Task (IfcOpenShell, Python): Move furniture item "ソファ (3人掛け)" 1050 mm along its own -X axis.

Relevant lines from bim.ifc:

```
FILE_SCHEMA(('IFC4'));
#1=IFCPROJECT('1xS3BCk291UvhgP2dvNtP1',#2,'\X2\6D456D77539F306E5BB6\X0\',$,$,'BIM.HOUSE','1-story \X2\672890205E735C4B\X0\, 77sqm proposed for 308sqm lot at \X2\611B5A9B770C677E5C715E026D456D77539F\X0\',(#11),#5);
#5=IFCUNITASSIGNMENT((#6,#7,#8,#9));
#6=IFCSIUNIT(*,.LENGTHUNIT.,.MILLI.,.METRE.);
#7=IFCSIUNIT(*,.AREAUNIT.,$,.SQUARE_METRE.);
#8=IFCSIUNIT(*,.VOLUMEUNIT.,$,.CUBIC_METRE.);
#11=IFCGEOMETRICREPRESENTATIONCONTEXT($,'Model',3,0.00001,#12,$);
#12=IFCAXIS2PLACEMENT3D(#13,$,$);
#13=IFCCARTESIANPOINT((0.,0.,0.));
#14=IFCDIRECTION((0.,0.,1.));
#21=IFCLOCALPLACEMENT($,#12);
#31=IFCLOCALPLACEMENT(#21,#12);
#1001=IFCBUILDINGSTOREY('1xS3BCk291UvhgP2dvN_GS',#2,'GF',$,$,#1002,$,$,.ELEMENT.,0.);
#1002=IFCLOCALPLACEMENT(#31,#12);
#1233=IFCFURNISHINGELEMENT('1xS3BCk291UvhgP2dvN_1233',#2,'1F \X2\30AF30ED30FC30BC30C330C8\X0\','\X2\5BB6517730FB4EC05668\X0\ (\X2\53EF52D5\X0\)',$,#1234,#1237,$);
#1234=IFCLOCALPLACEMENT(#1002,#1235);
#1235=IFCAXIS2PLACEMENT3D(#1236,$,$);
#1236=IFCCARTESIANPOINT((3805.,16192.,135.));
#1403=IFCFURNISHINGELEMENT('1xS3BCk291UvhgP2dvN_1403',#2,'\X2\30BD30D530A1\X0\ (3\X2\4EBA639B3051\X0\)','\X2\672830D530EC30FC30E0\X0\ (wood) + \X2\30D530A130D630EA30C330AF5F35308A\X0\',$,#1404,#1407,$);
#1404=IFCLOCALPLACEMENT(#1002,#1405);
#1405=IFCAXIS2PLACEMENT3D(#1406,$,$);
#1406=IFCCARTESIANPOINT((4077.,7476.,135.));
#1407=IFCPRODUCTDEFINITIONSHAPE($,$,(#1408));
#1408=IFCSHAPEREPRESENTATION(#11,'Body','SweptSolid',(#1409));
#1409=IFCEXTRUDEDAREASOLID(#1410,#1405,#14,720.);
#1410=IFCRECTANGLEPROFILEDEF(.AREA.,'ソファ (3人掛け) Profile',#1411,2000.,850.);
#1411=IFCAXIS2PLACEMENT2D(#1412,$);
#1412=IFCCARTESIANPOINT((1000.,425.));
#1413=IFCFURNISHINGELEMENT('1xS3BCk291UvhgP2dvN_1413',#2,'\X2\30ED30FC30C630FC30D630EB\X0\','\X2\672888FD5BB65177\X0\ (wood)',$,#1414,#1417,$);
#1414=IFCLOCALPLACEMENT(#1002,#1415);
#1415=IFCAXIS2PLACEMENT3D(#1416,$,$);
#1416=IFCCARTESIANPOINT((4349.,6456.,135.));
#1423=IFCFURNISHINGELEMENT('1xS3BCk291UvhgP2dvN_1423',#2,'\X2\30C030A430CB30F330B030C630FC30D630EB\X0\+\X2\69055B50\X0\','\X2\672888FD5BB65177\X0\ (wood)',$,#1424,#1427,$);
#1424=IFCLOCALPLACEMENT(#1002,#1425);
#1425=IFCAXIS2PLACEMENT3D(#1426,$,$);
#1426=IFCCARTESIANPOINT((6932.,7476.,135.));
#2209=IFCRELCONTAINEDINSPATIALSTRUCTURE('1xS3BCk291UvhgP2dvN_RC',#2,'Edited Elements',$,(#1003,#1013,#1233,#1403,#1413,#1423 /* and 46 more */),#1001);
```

```python
import ifcopenshell
import ifcopenshell.api.geometry
import ifcopenshell.util.placement
import ifcopenshell.util.unit

model = ifcopenshell.open("bim.ifc")
unit_scale = ifcopenshell.util.unit.calculate_unit_scale(model)

item = model.by_guid("1xS3BCk291UvhgP2dvN_1403")
matrix = ifcopenshell.util.placement.get_local_placement(item.ObjectPlacement)
matrix[:3, 3] -= matrix[:3, 0] * 1.05 / unit_scale
ifcopenshell.api.geometry.edit_object_placement(model, product=item, matrix=matrix, is_si=False)

print(ifcopenshell.util.placement.get_local_placement(item.ObjectPlacement).round(3) + 0.0)

model.write("bim_updated.ifc")
```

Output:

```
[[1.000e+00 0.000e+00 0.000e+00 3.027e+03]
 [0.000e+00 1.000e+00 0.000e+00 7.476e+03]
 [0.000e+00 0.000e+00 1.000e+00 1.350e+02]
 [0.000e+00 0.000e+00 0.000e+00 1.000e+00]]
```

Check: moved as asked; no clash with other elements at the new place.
